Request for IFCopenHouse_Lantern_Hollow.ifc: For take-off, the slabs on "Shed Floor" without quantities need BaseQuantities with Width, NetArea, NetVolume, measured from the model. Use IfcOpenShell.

First a look at what the model holds.

```python
import ifcopenshell
import ifcopenshell.util.element
import ifcopenshell.util.unit

model = ifcopenshell.open("IFCopenHouse_Lantern_Hollow.ifc")
print(model.schema)
for unit_type in ("LENGTHUNIT", "AREAUNIT", "VOLUMEUNIT"):
    print(unit_type, ifcopenshell.util.unit.calculate_unit_scale(model, unit_type))
storey = next(s for s in model.by_type("IfcBuildingStorey") if s.Name == "Shed Floor")
slabs = [e for e in ifcopenshell.util.element.get_decomposition(storey) if e.is_a("IfcSlab")]
for e in sorted(slabs, key=lambda e: e.id()):
    print(e.id(), e.is_a(), e.Name, list(ifcopenshell.util.element.get_psets(e, qtos_only=True)), sep=" | ")
```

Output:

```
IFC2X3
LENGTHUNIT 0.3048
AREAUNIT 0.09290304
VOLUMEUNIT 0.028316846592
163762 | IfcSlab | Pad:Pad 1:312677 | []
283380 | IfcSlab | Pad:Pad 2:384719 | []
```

```python
import ifcopenshell
import ifcopenshell.api.pset
import ifcopenshell.geom
import ifcopenshell.util.element
import ifcopenshell.util.shape
import ifcopenshell.util.unit

model = ifcopenshell.open("IFCopenHouse_Lantern_Hollow.ifc")
unit_scale = ifcopenshell.util.unit.calculate_unit_scale(model)
area_scale = ifcopenshell.util.unit.calculate_unit_scale(model, "AREAUNIT")
volume_scale = ifcopenshell.util.unit.calculate_unit_scale(model, "VOLUMEUNIT")
settings = ifcopenshell.geom.settings()

storey = next(s for s in model.by_type("IfcBuildingStorey") if s.Name == "Shed Floor")
slabs = [e for e in ifcopenshell.util.element.get_decomposition(storey) if e.is_a("IfcSlab")]

for e in sorted(slabs, key=lambda e: e.id()):
    if ifcopenshell.util.element.get_psets(e, qtos_only=True, should_inherit=False):
        continue
    # Geometry comes back in metres, in the element's own axes.
    shape = ifcopenshell.geom.create_shape(settings, e)
    values = {
        "Width": ifcopenshell.util.shape.get_z(shape.geometry) / unit_scale,
        "NetArea": ifcopenshell.util.shape.get_footprint_area(shape.geometry) / area_scale,
        "NetVolume": ifcopenshell.util.shape.get_volume(shape.geometry) / volume_scale,
    }
    qto = ifcopenshell.api.pset.add_qto(model, product=e, name="BaseQuantities")
    ifcopenshell.api.pset.edit_qto(model, qto=qto, properties=values)
    print(e.id(), {k: round(v, 3) for k, v in values.items()})

model.write("IFCopenHouse_Lantern_Hollow-out.ifc")
```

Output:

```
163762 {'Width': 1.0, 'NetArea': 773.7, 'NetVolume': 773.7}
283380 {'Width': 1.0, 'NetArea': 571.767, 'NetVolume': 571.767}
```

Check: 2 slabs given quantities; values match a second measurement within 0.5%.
